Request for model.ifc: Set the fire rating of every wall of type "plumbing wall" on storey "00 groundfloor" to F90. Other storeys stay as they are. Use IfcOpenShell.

First a look at what the model holds.

```python
import ifcopenshell
import ifcopenshell.util.element

model = ifcopenshell.open("model.ifc")
print(model.schema)
storey = next(s for s in model.by_type("IfcBuildingStorey") if s.Name == "00 groundfloor")
walls = [e for e in ifcopenshell.util.element.get_decomposition(storey) if e.is_a("IfcWall")]
seen = {}
for e in walls:
    element_type = ifcopenshell.util.element.get_type(e)
    key = (element_type.Name if element_type != e and element_type else None, ifcopenshell.util.element.get_pset(e, "Pset_WallCommon", "FireRating"))
    seen[key] = seen.get(key, 0) + 1
for (name, value), count in sorted(seen.items(), key=str):
    print(count, "x", name, "|", value)
```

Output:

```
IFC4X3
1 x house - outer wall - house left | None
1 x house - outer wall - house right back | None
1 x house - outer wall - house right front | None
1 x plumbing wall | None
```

```python
import ifcopenshell
import ifcopenshell.api.pset
import ifcopenshell.util.element

model = ifcopenshell.open("model.ifc")

storey = next(s for s in model.by_type("IfcBuildingStorey") if s.Name == "00 groundfloor")
walls = [e for e in ifcopenshell.util.element.get_decomposition(storey) if e.is_a("IfcWall")]

count = 0
for e in walls:
    element_type = ifcopenshell.util.element.get_type(e)
    if element_type in (None, e) or element_type.Name != "plumbing wall":
        continue
    # add_pset returns the element's existing set when there is one.
    pset = ifcopenshell.api.pset.add_pset(model, product=e, name="Pset_WallCommon")
    ifcopenshell.api.pset.edit_pset(model, pset=pset, properties={"FireRating": "F90"})
    count += 1

print(count, "walls updated")

model.write("model_edited.ifc")
```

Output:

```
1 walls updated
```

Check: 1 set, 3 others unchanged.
